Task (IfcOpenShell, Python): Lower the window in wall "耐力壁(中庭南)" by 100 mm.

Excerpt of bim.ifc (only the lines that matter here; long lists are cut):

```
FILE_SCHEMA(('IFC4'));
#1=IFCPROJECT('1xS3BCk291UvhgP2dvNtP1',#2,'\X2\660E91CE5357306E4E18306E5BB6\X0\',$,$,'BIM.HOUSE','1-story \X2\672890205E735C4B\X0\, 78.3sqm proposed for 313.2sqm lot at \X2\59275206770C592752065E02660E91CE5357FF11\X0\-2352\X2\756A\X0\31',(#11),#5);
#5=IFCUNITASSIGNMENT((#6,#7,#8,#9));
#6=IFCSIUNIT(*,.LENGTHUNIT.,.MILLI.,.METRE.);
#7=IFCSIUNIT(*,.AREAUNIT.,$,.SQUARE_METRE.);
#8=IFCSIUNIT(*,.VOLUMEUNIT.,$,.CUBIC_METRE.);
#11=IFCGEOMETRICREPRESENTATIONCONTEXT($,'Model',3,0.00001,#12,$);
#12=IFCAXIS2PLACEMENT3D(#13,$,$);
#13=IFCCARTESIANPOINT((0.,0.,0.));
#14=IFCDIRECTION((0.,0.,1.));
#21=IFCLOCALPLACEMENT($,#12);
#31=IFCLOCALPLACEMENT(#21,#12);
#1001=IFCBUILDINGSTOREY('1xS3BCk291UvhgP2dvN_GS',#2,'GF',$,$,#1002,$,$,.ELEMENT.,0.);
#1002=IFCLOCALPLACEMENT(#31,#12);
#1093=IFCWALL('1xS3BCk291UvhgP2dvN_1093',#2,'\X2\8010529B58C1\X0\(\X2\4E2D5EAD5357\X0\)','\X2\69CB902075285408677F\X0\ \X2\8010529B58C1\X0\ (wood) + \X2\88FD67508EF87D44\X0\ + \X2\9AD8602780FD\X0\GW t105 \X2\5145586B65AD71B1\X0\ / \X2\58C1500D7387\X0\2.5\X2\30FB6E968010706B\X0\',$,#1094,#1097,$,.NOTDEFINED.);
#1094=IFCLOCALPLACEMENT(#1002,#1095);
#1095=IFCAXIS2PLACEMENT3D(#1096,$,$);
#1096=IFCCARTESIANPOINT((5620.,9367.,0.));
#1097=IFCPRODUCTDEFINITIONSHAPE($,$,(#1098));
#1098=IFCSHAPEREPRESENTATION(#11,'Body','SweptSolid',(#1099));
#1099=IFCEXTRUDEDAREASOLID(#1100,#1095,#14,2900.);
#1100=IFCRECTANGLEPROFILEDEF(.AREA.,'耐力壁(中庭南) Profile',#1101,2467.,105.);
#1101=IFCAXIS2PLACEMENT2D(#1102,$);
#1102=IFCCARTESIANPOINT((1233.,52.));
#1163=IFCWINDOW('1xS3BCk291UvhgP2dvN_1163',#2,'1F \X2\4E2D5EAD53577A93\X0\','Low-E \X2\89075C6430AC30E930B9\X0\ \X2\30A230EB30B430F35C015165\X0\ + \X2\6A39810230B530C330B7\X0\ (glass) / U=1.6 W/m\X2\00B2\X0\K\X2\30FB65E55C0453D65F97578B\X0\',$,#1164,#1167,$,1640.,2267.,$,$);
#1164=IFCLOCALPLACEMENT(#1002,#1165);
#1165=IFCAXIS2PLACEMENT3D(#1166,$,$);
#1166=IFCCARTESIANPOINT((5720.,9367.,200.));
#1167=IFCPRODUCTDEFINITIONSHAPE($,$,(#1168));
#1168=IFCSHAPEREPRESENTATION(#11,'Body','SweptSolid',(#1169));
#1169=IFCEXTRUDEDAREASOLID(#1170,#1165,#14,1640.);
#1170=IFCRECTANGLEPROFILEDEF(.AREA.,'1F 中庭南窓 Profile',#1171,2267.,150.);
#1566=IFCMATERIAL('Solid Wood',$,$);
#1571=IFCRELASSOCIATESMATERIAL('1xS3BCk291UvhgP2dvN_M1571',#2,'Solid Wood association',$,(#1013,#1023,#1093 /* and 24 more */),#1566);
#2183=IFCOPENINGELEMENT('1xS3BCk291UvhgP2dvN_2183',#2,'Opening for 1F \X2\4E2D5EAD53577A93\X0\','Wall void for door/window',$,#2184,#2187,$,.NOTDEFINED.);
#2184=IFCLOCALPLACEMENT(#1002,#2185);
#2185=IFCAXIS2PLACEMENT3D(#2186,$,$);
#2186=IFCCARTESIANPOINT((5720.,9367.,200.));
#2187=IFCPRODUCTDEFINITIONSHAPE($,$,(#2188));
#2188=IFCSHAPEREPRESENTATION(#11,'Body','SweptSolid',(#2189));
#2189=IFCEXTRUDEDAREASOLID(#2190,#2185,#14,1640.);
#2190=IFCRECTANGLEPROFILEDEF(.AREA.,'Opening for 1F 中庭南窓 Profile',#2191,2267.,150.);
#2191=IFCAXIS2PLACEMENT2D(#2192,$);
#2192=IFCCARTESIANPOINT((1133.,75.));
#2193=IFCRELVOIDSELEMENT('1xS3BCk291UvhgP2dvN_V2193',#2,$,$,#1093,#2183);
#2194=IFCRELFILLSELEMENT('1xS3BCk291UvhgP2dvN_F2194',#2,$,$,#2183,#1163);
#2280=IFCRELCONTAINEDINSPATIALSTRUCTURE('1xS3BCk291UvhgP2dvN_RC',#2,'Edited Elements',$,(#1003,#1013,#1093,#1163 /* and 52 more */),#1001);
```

```python
import numpy as np
import ifcopenshell
import ifcopenshell.api.geometry
import ifcopenshell.util.placement
import ifcopenshell.util.unit

model = ifcopenshell.open("bim.ifc")
unit_scale = ifcopenshell.util.unit.calculate_unit_scale(model)

window = model.by_id(1163)
opening = window.FillsVoids[0].RelatingOpeningElement
dz = -100.0

shift = np.array([0.0, 0.0, dz])
# The window is not placed relative to its opening, so move both.
for product in (opening, window):
    matrix = ifcopenshell.util.placement.get_local_placement(product.ObjectPlacement)
    matrix[:3, 3] += shift
    ifcopenshell.api.geometry.edit_object_placement(model, product=product, matrix=matrix, is_si=False)

print(f"moved by {dz * unit_scale:+.3f} m")

model.write("bim_updated.ifc")
```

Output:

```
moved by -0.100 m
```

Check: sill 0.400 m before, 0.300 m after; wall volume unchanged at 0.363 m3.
